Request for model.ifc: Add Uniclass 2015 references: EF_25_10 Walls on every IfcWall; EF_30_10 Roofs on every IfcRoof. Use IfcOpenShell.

First a look at what the model holds.

```python
import ifcopenshell

model = ifcopenshell.open("model.ifc")
print(model.schema)
print("classifications:", [c.Name for c in model.by_type("IfcClassification")])
for ifc_class in ("IfcDoor", "IfcRoof", "IfcStair", "IfcWall", "IfcWindow"):
    print(ifc_class, len(model.by_type(ifc_class)))
```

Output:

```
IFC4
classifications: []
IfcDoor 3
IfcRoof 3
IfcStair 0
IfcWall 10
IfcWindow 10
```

```python
import ifcopenshell
import ifcopenshell.api.classification

model = ifcopenshell.open("model.ifc")

system = ifcopenshell.api.classification.add_classification(model, classification="Uniclass 2015")

codes = {
    "IfcWall": ("EF_25_10", "Walls"),
    "IfcRoof": ("EF_30_10", "Roofs"),
}
for ifc_class, (code, name) in codes.items():
    products = model.by_type(ifc_class)
    ifcopenshell.api.classification.add_reference(
        model, products=products, classification=system, identification=code, name=name
    )
    print(code, len(products))

model.write("model_updated.ifc")
```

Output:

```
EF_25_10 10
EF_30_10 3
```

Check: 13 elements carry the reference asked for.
